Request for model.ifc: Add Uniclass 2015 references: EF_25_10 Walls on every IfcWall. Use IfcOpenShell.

First a look at what the model holds.

```python
import ifcopenshell

model = ifcopenshell.open("model.ifc")
print(model.schema)
print("classifications:", [c.Name for c in model.by_type("IfcClassification")])
for ifc_class in ("IfcDoor", "IfcRoof", "IfcStair", "IfcWall", "IfcWindow"):
    print(ifc_class, len(model.by_type(ifc_class)))
```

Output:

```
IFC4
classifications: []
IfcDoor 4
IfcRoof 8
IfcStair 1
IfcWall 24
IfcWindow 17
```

```python
import ifcopenshell
import ifcopenshell.api.classification

model = ifcopenshell.open("model.ifc")

system = ifcopenshell.api.classification.add_classification(model, classification="Uniclass 2015")

codes = {
    "IfcWall": ("EF_25_10", "Walls"),
}
for ifc_class, (code, name) in codes.items():
    products = model.by_type(ifc_class)
    ifcopenshell.api.classification.add_reference(
        model, products=products, classification=system, identification=code, name=name
    )
    print(code, len(products))

model.write("model_rev.ifc")
```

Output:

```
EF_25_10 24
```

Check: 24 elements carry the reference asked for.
